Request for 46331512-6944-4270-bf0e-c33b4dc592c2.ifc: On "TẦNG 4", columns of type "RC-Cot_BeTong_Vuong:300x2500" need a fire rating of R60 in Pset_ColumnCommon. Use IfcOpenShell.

First a look at what the model holds.

```python
import ifcopenshell
import ifcopenshell.util.element

model = ifcopenshell.open("46331512-6944-4270-bf0e-c33b4dc592c2.ifc")
print(model.schema)
storey = next(s for s in model.by_type("IfcBuildingStorey") if s.Name == "TẦNG 4")
columns = [e for e in ifcopenshell.util.element.get_decomposition(storey) if e.is_a("IfcColumn")]
seen = {}
for e in columns:
    element_type = ifcopenshell.util.element.get_type(e)
    key = (element_type.Name if element_type != e and element_type else None, ifcopenshell.util.element.get_pset(e, "Pset_ColumnCommon", "FireRating"))
    seen[key] = seen.get(key, 0) + 1
for (name, value), count in sorted(seen.items(), key=str):
    print(count, "x", name, "|", value)
```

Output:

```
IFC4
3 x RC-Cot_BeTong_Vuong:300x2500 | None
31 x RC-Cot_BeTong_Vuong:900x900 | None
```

```python
import ifcopenshell
import ifcopenshell.api.pset
import ifcopenshell.util.element

model = ifcopenshell.open("46331512-6944-4270-bf0e-c33b4dc592c2.ifc")

storey = next(s for s in model.by_type("IfcBuildingStorey") if s.Name == "TẦNG 4")
columns = [e for e in ifcopenshell.util.element.get_decomposition(storey) if e.is_a("IfcColumn")]

count = 0
for e in columns:
    element_type = ifcopenshell.util.element.get_type(e)
    if element_type in (None, e) or element_type.Name != "RC-Cot_BeTong_Vuong:300x2500":
        continue
    # add_pset returns the element's existing set when there is one.
    pset = ifcopenshell.api.pset.add_pset(model, product=e, name="Pset_ColumnCommon")
    ifcopenshell.api.pset.edit_pset(model, pset=pset, properties={"FireRating": "R60"})
    count += 1

print(count, "columns updated")

model.write("46331512-6944-4270-bf0e-c33b4dc592c2_rev.ifc")
```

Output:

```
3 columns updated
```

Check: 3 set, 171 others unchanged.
